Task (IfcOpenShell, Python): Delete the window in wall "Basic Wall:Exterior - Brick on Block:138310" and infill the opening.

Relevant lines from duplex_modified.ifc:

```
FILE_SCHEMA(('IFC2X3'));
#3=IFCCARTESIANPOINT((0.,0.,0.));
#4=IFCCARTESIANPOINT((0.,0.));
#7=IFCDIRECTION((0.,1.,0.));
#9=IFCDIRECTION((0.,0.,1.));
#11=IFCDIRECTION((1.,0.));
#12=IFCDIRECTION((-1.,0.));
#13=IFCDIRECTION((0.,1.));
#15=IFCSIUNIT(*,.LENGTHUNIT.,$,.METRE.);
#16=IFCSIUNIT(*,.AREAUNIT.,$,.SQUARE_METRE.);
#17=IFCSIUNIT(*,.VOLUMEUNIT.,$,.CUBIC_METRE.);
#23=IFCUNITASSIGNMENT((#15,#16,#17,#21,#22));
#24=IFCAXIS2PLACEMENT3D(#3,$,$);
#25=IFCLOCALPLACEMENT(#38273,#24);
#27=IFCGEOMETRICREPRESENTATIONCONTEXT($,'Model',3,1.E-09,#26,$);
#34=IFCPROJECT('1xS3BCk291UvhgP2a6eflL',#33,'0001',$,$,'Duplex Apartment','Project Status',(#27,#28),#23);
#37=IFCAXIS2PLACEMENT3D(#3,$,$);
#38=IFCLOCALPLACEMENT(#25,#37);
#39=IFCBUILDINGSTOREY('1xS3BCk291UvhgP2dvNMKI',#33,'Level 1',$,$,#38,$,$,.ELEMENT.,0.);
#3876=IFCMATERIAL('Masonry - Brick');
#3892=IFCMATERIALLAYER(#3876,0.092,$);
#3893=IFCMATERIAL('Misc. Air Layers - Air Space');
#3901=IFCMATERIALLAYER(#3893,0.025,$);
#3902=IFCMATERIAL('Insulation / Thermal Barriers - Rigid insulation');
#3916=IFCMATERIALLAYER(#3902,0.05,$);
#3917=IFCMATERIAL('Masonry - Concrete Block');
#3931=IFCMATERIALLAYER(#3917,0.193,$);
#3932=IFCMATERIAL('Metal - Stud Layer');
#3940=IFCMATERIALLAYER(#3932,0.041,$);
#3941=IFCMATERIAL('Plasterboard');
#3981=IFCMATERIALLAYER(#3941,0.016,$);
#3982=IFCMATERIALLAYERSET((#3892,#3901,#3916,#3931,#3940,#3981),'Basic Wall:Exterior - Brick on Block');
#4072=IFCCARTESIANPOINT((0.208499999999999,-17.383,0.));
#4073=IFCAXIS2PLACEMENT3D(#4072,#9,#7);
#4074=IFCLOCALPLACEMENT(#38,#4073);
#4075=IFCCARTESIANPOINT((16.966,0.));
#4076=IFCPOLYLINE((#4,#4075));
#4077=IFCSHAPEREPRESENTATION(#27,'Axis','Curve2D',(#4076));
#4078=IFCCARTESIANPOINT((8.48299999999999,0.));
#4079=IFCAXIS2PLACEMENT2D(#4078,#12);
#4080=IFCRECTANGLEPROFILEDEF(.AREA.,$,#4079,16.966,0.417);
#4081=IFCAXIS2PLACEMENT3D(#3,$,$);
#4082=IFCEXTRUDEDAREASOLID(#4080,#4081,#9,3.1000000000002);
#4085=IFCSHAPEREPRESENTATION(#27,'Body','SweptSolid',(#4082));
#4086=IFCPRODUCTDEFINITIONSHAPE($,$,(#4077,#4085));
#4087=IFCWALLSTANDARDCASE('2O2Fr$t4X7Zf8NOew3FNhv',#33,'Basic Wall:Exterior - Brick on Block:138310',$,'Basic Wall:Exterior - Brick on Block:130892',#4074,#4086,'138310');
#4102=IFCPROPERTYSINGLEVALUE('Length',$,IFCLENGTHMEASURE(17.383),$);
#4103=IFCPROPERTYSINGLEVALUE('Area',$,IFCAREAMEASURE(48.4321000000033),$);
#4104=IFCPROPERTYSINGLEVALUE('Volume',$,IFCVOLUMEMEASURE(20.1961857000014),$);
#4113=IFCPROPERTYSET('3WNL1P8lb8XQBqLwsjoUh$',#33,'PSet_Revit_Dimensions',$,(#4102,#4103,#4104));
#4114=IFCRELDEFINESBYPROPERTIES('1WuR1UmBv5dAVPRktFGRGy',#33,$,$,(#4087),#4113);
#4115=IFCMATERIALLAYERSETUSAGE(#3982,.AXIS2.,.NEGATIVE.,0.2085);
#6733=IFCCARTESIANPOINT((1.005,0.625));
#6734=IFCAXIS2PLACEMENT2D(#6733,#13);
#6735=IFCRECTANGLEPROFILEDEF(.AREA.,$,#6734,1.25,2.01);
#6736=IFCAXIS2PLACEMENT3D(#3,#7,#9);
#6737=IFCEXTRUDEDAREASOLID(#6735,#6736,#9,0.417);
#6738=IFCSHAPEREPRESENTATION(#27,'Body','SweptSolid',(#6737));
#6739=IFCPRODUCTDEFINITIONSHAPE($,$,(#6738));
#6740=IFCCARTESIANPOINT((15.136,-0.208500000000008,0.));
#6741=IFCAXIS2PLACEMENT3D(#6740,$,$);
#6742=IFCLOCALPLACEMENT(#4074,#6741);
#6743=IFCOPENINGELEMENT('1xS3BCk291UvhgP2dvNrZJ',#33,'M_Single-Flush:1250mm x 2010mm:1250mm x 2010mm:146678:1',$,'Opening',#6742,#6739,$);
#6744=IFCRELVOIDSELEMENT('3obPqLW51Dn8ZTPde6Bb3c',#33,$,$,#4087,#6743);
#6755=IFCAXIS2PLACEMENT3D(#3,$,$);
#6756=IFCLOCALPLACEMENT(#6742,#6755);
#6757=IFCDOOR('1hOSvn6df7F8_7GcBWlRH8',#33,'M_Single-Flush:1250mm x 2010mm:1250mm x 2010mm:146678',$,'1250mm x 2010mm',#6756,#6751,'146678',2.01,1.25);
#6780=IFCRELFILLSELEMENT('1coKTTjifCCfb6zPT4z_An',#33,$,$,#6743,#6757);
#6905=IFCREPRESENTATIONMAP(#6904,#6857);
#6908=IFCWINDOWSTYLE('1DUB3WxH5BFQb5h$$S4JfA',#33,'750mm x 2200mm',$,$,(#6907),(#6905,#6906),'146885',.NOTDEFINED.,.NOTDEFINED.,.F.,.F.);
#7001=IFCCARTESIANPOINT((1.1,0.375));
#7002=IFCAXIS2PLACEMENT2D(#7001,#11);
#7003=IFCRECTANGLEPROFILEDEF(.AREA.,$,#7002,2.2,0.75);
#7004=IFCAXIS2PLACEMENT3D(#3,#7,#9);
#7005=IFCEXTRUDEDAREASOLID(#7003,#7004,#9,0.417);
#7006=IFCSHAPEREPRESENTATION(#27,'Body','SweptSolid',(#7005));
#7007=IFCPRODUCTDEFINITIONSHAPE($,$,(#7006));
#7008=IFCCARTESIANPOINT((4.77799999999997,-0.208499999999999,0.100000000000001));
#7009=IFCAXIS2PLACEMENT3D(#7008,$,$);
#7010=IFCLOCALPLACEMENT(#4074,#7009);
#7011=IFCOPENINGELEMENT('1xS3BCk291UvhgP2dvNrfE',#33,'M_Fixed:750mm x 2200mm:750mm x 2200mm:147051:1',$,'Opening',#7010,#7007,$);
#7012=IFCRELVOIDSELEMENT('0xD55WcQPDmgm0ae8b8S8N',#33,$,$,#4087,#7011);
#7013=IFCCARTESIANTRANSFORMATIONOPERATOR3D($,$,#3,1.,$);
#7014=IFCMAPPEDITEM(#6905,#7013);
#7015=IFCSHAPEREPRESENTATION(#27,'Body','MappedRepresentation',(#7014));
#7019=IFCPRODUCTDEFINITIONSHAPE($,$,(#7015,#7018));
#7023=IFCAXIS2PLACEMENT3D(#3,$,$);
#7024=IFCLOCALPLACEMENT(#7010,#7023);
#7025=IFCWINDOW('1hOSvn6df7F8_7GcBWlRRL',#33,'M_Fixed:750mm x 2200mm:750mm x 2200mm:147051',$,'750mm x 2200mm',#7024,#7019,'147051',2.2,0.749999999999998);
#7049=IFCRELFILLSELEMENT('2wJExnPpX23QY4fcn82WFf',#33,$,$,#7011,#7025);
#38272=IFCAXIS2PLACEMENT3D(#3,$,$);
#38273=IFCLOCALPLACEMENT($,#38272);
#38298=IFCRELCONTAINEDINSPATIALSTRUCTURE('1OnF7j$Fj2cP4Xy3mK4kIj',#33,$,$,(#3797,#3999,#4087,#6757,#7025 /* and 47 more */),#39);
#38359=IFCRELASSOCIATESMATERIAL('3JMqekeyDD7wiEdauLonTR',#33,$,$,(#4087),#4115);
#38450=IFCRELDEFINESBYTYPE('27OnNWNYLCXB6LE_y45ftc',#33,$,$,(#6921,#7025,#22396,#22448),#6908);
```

```python
import ifcopenshell
import ifcopenshell.api.feature
import ifcopenshell.api.pset
import ifcopenshell.api.root
import ifcopenshell.geom
import ifcopenshell.util.element
import ifcopenshell.util.shape
import ifcopenshell.util.unit

model = ifcopenshell.open("duplex_modified.ifc")
area_scale = ifcopenshell.util.unit.calculate_unit_scale(model, "AREAUNIT")
volume_scale = ifcopenshell.util.unit.calculate_unit_scale(model, "VOLUMEUNIT")
settings = ifcopenshell.geom.settings()


def volume(element):
    """Net volume in cubic metres, openings subtracted."""
    shape = ifcopenshell.geom.create_shape(settings, element)
    return ifcopenshell.util.shape.get_volume(shape.geometry)


window = model.by_id(7025)
opening = window.FillsVoids[0].RelatingOpeningElement
wall = opening.VoidsElements[0].RelatingBuildingElement
before = volume(wall)

ifcopenshell.api.root.remove_product(model, product=window)
ifcopenshell.api.feature.remove_feature(model, feature=opening)

after = volume(wall)
thickness = 0.417  # wall thickness in metres

# Update the wall's stored quantities.
pset = model.by_id(ifcopenshell.util.element.get_pset(wall, "PSet_Revit_Dimensions", should_inherit=False)["id"])
ifcopenshell.api.pset.edit_pset(model, pset=pset, properties={
    "Area": model.create_entity("IfcAreaMeasure", after / thickness / area_scale),
    "Volume": model.create_entity("IfcVolumeMeasure", after / volume_scale),
})

print(f"wall volume {before:.3f} -> {after:.3f} m3")

model.write("duplex_modified-out.ifc")
```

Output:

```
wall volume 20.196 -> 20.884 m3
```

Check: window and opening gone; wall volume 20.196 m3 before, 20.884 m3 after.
